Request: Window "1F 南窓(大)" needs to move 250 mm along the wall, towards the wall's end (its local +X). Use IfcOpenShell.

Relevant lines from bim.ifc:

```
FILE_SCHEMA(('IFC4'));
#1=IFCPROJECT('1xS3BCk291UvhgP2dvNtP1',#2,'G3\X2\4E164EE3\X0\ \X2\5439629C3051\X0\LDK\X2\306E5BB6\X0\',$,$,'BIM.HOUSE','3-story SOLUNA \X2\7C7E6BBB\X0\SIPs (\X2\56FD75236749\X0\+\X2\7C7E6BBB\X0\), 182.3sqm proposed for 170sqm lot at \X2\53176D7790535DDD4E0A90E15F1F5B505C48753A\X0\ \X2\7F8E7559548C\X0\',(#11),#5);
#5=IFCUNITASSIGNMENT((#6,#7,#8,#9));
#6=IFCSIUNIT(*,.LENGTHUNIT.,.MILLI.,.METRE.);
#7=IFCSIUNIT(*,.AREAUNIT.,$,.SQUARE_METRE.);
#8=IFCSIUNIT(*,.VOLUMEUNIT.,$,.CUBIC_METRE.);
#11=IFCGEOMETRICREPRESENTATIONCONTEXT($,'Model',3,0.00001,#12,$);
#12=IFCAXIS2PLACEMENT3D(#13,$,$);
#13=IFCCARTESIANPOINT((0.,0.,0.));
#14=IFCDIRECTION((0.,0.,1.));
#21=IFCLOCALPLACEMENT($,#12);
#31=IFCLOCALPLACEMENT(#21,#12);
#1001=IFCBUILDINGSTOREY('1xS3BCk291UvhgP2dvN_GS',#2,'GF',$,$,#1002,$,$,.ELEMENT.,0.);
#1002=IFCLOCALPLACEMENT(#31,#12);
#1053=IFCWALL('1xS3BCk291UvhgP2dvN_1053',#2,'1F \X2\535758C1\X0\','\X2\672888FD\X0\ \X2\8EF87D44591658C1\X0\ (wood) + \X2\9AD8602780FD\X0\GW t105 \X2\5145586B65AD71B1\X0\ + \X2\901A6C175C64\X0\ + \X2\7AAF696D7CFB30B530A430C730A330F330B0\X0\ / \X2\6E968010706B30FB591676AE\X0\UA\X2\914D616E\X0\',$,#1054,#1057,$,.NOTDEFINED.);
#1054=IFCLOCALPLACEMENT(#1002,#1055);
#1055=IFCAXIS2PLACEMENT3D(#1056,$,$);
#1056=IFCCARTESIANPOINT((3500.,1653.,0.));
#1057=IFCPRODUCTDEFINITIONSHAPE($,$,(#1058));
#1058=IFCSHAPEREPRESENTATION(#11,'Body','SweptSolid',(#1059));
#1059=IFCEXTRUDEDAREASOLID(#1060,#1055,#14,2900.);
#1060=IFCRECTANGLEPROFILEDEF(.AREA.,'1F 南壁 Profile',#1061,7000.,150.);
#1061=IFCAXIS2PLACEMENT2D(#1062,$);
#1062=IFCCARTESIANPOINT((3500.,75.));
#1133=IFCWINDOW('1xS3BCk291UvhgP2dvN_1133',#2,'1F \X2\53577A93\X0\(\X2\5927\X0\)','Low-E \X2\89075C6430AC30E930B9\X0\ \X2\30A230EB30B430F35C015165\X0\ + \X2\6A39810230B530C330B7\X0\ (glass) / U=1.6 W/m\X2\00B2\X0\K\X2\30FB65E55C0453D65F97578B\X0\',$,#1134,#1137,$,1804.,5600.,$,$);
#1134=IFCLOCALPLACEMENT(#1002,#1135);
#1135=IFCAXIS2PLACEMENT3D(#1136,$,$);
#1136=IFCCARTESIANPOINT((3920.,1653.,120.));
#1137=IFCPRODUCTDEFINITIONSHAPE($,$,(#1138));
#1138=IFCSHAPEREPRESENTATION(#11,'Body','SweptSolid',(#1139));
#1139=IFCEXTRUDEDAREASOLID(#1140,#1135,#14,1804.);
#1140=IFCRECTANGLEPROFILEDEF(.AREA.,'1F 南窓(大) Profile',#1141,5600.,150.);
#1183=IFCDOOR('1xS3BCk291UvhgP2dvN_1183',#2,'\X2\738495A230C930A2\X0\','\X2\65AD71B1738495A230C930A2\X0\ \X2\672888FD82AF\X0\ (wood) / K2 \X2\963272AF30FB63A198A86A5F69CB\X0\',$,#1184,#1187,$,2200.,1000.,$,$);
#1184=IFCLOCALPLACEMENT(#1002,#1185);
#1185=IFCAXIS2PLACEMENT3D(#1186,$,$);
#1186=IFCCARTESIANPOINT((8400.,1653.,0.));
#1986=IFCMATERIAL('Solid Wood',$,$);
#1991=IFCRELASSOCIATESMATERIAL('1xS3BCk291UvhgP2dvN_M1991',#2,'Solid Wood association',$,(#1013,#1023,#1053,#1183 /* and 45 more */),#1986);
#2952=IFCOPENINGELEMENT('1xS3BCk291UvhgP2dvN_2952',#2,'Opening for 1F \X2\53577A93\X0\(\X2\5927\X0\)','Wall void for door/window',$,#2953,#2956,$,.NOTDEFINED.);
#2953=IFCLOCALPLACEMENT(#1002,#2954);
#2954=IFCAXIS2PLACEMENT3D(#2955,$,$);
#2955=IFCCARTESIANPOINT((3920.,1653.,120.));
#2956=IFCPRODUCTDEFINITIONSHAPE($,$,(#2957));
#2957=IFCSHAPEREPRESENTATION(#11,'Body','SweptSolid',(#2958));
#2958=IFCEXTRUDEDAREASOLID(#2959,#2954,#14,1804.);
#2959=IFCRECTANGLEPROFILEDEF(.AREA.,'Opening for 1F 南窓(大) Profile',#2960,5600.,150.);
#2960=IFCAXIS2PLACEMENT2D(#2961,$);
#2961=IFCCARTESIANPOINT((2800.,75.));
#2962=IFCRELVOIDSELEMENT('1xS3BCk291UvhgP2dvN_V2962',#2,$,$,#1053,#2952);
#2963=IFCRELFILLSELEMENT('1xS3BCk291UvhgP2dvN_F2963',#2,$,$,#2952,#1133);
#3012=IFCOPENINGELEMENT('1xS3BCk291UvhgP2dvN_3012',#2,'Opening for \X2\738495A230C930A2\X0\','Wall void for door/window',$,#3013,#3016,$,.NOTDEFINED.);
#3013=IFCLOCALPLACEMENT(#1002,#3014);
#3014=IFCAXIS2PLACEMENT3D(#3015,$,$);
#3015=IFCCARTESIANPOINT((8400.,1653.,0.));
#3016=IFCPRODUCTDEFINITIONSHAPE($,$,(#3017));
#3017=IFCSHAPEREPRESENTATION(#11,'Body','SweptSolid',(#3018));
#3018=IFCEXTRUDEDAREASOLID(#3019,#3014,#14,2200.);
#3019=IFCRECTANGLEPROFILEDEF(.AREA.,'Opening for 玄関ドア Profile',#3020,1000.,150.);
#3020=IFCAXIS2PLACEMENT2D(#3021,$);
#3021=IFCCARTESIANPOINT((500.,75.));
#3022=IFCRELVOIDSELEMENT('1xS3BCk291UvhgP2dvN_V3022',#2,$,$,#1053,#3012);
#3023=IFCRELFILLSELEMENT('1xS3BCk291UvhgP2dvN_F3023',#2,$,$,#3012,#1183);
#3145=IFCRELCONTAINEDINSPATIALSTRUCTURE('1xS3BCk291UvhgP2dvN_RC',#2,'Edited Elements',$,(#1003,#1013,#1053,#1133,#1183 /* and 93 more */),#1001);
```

```python
import ifcopenshell
import ifcopenshell.api.geometry
import ifcopenshell.util.placement
import ifcopenshell.util.unit

model = ifcopenshell.open("bim.ifc")
unit_scale = ifcopenshell.util.unit.calculate_unit_scale(model)

window = model.by_guid("1xS3BCk291UvhgP2dvN_1133")
opening = window.FillsVoids[0].RelatingOpeningElement
wall = opening.VoidsElements[0].RelatingBuildingElement

wall_matrix = ifcopenshell.util.placement.get_local_placement(wall.ObjectPlacement)
shift = wall_matrix[:3, 0] * 0.25 / unit_scale
before = ifcopenshell.util.placement.get_local_placement(window.ObjectPlacement)[:3, 3].copy()

# The window is not placed relative to its opening, so move both.
for product in (opening, window):
    matrix = ifcopenshell.util.placement.get_local_placement(product.ObjectPlacement)
    matrix[:3, 3] += shift
    ifcopenshell.api.geometry.edit_object_placement(model, product=product, matrix=matrix, is_si=False)

after = ifcopenshell.util.placement.get_local_placement(window.ObjectPlacement)[:3, 3]
print("window moved by", (after - before).round(3) + 0.0)

model.write("bim_rev.ifc")
```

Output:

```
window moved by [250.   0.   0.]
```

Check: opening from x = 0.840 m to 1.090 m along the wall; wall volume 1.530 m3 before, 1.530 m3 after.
